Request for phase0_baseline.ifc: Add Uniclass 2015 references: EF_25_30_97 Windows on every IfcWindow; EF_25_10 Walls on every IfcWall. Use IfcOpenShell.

First a look at what the model holds.

```python
import ifcopenshell

model = ifcopenshell.open("phase0_baseline.ifc")
print(model.schema)
print("classifications:", [c.Name for c in model.by_type("IfcClassification")])
for ifc_class in ("IfcDoor", "IfcRoof", "IfcStair", "IfcWall", "IfcWindow"):
    print(ifc_class, len(model.by_type(ifc_class)))
```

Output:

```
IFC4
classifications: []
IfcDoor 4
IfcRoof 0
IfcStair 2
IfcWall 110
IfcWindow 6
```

```python
import ifcopenshell
import ifcopenshell.api.classification

model = ifcopenshell.open("phase0_baseline.ifc")

system = ifcopenshell.api.classification.add_classification(model, classification="Uniclass 2015")

codes = {
    "IfcWindow": ("EF_25_30_97", "Windows"),
    "IfcWall": ("EF_25_10", "Walls"),
}
for ifc_class, (code, name) in codes.items():
    products = model.by_type(ifc_class)
    ifcopenshell.api.classification.add_reference(
        model, products=products, classification=system, identification=code, name=name
    )
    print(code, len(products))

model.write("phase0_baseline_edited.ifc")
```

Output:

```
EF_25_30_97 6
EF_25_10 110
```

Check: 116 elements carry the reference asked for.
